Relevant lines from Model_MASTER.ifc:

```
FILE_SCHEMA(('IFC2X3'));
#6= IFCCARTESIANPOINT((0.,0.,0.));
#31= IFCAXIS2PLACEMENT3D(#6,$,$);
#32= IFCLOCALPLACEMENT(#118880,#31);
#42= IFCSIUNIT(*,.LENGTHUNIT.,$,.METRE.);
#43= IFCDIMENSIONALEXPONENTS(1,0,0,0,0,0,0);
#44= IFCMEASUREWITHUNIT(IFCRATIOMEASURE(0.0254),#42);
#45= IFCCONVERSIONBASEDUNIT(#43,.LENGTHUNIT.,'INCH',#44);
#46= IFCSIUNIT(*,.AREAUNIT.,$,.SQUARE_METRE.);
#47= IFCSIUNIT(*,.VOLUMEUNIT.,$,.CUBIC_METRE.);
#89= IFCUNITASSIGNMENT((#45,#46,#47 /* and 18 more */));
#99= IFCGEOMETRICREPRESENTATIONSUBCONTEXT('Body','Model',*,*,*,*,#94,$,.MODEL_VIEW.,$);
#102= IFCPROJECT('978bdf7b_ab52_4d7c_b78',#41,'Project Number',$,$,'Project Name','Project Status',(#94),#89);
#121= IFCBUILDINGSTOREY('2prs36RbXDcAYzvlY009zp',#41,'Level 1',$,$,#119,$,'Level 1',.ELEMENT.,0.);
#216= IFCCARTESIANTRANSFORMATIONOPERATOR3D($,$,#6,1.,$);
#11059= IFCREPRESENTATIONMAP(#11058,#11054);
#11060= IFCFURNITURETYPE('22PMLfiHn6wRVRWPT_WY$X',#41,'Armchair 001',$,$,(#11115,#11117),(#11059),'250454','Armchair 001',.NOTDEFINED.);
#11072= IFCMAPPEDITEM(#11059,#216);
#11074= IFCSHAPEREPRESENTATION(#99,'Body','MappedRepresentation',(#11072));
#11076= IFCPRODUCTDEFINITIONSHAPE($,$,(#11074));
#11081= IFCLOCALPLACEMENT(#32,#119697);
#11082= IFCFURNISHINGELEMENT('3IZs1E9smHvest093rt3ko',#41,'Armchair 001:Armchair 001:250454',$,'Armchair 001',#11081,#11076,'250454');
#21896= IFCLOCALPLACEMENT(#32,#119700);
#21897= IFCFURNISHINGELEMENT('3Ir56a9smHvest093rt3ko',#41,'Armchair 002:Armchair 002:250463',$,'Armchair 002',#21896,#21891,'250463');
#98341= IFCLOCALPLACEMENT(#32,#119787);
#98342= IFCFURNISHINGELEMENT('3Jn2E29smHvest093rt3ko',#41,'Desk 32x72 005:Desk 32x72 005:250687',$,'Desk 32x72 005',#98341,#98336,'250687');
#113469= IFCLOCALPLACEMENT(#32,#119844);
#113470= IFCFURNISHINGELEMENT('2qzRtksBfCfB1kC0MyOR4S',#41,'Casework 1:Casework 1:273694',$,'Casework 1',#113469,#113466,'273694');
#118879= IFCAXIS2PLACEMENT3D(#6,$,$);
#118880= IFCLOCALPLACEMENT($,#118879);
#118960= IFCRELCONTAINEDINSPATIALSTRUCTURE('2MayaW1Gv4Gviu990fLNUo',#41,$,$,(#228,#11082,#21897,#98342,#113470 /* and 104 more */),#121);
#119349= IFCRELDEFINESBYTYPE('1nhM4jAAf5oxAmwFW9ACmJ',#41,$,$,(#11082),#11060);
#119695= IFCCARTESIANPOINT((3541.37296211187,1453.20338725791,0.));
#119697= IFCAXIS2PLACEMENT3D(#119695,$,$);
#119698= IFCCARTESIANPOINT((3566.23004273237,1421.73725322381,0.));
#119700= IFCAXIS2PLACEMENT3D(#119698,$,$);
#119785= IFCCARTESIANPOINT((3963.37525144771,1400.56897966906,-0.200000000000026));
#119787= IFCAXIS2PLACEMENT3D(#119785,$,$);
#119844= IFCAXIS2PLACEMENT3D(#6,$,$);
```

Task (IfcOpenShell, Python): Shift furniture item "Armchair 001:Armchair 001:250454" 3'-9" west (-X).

```python
import ifcopenshell
import ifcopenshell.api.geometry
import ifcopenshell.util.placement
import ifcopenshell.util.unit

model = ifcopenshell.open("Model_MASTER.ifc")
unit_scale = ifcopenshell.util.unit.calculate_unit_scale(model)

item = model.by_guid("3IZs1E9smHvest093rt3ko")
matrix = ifcopenshell.util.placement.get_local_placement(item.ObjectPlacement)
matrix[0, 3] -= 45 * 0.0254 / unit_scale
ifcopenshell.api.geometry.edit_object_placement(model, product=item, matrix=matrix, is_si=False)

print(ifcopenshell.util.placement.get_local_placement(item.ObjectPlacement).round(3) + 0.0)

model.write("Model_MASTER_edited.ifc")
```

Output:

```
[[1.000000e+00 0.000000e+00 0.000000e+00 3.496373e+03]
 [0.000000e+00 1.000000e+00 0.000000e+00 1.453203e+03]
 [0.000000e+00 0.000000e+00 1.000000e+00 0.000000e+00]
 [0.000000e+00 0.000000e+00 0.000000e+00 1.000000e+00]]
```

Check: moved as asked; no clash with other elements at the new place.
